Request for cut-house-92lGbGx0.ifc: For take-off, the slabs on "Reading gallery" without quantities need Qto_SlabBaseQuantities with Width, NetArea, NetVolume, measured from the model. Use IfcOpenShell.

First a look at what the model holds.

```python
import ifcopenshell
import ifcopenshell.util.element
import ifcopenshell.util.unit

model = ifcopenshell.open("cut-house-92lGbGx0.ifc")
print(model.schema)
for unit_type in ("LENGTHUNIT", "AREAUNIT", "VOLUMEUNIT"):
    print(unit_type, ifcopenshell.util.unit.calculate_unit_scale(model, unit_type))
storey = next(s for s in model.by_type("IfcBuildingStorey") if s.Name == "Reading gallery")
slabs = [e for e in ifcopenshell.util.element.get_decomposition(storey) if e.is_a("IfcSlab")]
for e in sorted(slabs, key=lambda e: e.id()):
    print(e.id(), e.is_a(), e.Name, list(ifcopenshell.util.element.get_psets(e, qtos_only=True)), sep=" | ")
```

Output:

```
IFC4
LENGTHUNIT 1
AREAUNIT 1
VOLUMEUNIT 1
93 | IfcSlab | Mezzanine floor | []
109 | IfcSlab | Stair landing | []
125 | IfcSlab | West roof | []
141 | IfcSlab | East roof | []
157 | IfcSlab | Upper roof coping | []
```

```python
import ifcopenshell
import ifcopenshell.api.pset
import ifcopenshell.geom
import ifcopenshell.util.element
import ifcopenshell.util.shape
import ifcopenshell.util.unit

model = ifcopenshell.open("cut-house-92lGbGx0.ifc")
unit_scale = ifcopenshell.util.unit.calculate_unit_scale(model)
area_scale = ifcopenshell.util.unit.calculate_unit_scale(model, "AREAUNIT")
volume_scale = ifcopenshell.util.unit.calculate_unit_scale(model, "VOLUMEUNIT")
settings = ifcopenshell.geom.settings()

storey = next(s for s in model.by_type("IfcBuildingStorey") if s.Name == "Reading gallery")
slabs = [e for e in ifcopenshell.util.element.get_decomposition(storey) if e.is_a("IfcSlab")]

for e in sorted(slabs, key=lambda e: e.id()):
    if ifcopenshell.util.element.get_psets(e, qtos_only=True, should_inherit=False):
        continue
    # Geometry comes back in metres, in the element's own axes.
    shape = ifcopenshell.geom.create_shape(settings, e)
    values = {
        "Width": ifcopenshell.util.shape.get_z(shape.geometry) / unit_scale,
        "NetArea": ifcopenshell.util.shape.get_footprint_area(shape.geometry) / area_scale,
        "NetVolume": ifcopenshell.util.shape.get_volume(shape.geometry) / volume_scale,
    }
    qto = ifcopenshell.api.pset.add_qto(model, product=e, name="Qto_SlabBaseQuantities")
    ifcopenshell.api.pset.edit_qto(model, qto=qto, properties=values)
    print(e.id(), {k: round(v, 3) for k, v in values.items()})

model.write("cut-house-92lGbGx0_edited.ifc")
```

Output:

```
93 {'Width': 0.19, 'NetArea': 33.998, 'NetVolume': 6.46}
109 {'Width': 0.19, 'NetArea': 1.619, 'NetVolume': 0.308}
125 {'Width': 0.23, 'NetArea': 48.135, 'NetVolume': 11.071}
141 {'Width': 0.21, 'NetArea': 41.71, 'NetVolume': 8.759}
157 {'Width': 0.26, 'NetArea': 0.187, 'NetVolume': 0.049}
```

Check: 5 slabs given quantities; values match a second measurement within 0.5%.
